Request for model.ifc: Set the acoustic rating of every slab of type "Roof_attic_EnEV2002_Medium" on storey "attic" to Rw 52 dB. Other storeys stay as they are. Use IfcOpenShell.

First a look at what the model holds.

```python
import ifcopenshell
import ifcopenshell.util.element

model = ifcopenshell.open("model.ifc")
print(model.schema)
storey = next(s for s in model.by_type("IfcBuildingStorey") if s.Name == "attic")
slabs = [e for e in ifcopenshell.util.element.get_decomposition(storey) if e.is_a("IfcSlab")]
seen = {}
for e in slabs:
    element_type = ifcopenshell.util.element.get_type(e)
    key = (element_type.Name if element_type != e and element_type else None, ifcopenshell.util.element.get_pset(e, "Pset_SlabCommon", "AcousticRating"))
    seen[key] = seen.get(key, 0) + 1
for (name, value), count in sorted(seen.items(), key=str):
    print(count, "x", name, "|", value)
```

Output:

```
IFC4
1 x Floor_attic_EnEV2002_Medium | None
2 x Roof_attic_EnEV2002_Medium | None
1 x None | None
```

```python
import ifcopenshell
import ifcopenshell.api.pset
import ifcopenshell.util.element

model = ifcopenshell.open("model.ifc")

storey = next(s for s in model.by_type("IfcBuildingStorey") if s.Name == "attic")
slabs = [e for e in ifcopenshell.util.element.get_decomposition(storey) if e.is_a("IfcSlab")]

count = 0
for e in slabs:
    element_type = ifcopenshell.util.element.get_type(e)
    if element_type in (None, e) or element_type.Name != "Roof_attic_EnEV2002_Medium":
        continue
    # add_pset returns the element's existing set when there is one.
    pset = ifcopenshell.api.pset.add_pset(model, product=e, name="Pset_SlabCommon")
    ifcopenshell.api.pset.edit_pset(model, pset=pset, properties={"AcousticRating": "Rw 52 dB"})
    count += 1

print(count, "slabs updated")

model.write("model_v2.ifc")
```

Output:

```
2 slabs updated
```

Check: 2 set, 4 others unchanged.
